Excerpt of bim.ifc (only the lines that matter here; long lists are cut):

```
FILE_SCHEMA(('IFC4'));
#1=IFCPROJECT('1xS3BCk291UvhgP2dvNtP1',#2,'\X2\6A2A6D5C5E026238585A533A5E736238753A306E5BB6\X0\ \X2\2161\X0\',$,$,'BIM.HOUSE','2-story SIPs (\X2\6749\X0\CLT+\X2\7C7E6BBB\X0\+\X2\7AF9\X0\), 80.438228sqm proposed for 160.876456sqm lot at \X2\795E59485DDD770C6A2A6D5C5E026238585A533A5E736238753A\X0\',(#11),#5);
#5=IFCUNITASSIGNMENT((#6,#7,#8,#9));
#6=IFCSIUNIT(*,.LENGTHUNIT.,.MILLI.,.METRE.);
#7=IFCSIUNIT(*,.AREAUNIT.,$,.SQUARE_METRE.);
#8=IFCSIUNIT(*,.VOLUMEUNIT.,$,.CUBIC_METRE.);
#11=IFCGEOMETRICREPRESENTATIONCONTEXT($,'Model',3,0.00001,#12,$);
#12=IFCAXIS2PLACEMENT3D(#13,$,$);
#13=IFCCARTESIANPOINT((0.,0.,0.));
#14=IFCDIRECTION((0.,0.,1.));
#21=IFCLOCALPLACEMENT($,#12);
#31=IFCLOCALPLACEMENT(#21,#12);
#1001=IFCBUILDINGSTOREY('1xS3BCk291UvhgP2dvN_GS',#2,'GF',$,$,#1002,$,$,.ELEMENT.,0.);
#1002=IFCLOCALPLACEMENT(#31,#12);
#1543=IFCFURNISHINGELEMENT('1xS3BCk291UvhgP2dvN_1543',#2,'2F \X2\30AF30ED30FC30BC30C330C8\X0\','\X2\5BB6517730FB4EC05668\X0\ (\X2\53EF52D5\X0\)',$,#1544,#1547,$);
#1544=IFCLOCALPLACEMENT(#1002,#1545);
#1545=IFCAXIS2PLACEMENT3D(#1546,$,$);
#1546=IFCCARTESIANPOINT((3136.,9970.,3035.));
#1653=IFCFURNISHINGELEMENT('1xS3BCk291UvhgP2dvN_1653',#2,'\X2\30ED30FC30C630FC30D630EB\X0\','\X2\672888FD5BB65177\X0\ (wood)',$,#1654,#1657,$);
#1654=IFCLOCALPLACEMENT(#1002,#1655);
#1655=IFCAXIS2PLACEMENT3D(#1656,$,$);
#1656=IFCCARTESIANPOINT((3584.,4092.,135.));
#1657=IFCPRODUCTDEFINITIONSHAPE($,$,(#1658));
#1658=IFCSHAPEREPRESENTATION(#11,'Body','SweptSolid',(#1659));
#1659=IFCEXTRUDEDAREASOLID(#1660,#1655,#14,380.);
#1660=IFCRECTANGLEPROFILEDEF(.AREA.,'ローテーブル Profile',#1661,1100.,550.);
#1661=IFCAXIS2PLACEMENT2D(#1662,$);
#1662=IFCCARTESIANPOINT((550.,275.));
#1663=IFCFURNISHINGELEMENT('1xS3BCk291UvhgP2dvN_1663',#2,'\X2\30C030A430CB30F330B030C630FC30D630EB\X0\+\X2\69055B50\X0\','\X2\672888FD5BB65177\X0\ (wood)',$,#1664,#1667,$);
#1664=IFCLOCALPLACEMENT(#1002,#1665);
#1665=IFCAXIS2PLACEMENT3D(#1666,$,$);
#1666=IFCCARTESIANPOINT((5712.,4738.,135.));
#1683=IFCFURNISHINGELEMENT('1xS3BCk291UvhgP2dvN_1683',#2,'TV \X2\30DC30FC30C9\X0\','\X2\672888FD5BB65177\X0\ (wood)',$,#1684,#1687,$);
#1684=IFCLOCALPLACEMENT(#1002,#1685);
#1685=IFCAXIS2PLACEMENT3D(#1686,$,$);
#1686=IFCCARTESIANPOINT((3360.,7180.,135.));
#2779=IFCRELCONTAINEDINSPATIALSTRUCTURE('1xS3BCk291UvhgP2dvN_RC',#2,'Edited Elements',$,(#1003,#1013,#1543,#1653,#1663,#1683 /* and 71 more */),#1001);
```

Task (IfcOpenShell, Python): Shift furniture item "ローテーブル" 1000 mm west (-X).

```python
import ifcopenshell
import ifcopenshell.api.geometry
import ifcopenshell.util.placement
import ifcopenshell.util.unit

model = ifcopenshell.open("bim.ifc")
unit_scale = ifcopenshell.util.unit.calculate_unit_scale(model)

item = model.by_guid("1xS3BCk291UvhgP2dvN_1653")
matrix = ifcopenshell.util.placement.get_local_placement(item.ObjectPlacement)
matrix[0, 3] -= 1 / unit_scale
ifcopenshell.api.geometry.edit_object_placement(model, product=item, matrix=matrix, is_si=False)

print(ifcopenshell.util.placement.get_local_placement(item.ObjectPlacement).round(3) + 0.0)

model.write("bim_v2.ifc")
```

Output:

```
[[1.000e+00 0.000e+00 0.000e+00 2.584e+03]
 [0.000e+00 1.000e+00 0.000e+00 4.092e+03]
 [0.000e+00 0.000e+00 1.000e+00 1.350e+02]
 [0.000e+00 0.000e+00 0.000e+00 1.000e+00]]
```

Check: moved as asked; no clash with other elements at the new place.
